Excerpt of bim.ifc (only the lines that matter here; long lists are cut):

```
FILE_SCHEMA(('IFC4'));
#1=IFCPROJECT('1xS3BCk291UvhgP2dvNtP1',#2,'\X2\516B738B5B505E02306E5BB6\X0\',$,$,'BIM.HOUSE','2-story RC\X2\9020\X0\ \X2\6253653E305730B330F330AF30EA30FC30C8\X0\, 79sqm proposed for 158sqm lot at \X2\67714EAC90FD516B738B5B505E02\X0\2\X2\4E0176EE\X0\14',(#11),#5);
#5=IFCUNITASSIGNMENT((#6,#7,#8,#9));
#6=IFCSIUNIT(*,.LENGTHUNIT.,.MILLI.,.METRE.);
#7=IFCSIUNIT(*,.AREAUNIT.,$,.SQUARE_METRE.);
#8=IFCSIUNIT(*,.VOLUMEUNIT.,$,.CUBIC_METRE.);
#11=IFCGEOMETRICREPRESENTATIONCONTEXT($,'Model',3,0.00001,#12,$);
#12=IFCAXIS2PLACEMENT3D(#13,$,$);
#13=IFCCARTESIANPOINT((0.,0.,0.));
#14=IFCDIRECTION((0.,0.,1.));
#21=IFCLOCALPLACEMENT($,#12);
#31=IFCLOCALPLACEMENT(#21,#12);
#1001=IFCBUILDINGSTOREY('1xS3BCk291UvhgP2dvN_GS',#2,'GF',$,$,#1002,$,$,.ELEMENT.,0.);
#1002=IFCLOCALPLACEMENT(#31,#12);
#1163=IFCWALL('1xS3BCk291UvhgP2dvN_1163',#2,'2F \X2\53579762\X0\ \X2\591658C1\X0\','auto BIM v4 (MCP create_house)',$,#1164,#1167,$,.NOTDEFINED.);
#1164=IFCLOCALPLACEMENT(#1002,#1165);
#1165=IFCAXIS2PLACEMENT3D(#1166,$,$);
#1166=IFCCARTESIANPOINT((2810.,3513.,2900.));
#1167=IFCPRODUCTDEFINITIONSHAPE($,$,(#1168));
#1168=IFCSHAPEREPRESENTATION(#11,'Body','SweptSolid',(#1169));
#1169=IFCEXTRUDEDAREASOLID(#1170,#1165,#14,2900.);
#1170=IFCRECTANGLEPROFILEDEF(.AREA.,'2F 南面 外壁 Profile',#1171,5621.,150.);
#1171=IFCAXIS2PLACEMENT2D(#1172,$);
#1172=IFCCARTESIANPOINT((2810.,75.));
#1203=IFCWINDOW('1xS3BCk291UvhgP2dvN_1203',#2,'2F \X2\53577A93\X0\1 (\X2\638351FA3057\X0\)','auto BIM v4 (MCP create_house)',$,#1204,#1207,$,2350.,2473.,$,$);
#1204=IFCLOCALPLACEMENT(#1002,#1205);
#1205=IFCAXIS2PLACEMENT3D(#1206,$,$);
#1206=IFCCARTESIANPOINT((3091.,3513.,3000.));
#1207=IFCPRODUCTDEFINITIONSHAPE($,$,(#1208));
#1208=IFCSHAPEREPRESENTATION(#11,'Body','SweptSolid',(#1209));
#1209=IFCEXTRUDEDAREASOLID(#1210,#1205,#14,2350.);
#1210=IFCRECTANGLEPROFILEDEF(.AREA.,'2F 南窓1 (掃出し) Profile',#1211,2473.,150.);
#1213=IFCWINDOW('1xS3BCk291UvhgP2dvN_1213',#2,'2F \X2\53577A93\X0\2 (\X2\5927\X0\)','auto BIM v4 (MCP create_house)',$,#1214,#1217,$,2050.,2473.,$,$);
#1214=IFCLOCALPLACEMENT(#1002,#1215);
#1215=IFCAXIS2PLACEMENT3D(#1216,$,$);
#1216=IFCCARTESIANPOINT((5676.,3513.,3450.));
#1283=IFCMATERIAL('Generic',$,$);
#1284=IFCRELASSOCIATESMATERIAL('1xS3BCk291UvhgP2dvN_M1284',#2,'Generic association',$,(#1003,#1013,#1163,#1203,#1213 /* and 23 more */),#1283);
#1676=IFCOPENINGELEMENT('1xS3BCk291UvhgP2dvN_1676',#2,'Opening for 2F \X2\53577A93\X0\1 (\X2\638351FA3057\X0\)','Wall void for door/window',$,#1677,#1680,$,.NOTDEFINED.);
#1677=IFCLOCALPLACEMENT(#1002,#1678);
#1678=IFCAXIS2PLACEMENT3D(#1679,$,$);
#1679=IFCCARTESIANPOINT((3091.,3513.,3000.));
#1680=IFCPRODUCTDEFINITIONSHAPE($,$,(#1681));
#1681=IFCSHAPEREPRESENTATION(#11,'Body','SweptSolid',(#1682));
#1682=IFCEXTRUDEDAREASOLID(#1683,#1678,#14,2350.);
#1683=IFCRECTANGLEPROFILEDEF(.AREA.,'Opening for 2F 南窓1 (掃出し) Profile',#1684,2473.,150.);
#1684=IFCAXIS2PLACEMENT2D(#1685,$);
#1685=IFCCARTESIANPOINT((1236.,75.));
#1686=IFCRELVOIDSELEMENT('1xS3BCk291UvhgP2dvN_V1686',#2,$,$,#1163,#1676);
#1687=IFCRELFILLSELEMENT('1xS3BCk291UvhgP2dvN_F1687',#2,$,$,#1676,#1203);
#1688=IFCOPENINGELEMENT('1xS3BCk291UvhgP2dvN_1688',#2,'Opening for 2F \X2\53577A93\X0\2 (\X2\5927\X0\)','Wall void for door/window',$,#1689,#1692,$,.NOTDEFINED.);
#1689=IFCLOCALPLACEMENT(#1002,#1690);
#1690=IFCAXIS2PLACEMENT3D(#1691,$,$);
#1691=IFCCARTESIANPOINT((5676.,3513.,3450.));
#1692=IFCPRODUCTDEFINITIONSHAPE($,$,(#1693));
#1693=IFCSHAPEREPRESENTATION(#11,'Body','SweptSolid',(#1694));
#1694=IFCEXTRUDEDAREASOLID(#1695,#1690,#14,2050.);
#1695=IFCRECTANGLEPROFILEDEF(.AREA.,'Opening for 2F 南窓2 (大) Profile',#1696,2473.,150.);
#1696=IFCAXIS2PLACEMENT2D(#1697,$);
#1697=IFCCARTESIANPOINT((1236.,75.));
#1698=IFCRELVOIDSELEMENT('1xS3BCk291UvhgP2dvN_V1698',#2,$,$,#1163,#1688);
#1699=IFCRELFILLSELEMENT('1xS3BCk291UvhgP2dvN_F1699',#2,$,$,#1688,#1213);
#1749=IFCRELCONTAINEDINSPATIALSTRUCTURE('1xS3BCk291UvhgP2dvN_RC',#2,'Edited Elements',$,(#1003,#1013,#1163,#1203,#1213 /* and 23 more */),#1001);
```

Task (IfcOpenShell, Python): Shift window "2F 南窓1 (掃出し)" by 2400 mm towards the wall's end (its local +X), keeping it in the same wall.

```python
import ifcopenshell
import ifcopenshell.api.geometry
import ifcopenshell.util.placement
import ifcopenshell.util.unit

model = ifcopenshell.open("bim.ifc")
unit_scale = ifcopenshell.util.unit.calculate_unit_scale(model)

window = model.by_guid("1xS3BCk291UvhgP2dvN_1203")
opening = window.FillsVoids[0].RelatingOpeningElement
wall = opening.VoidsElements[0].RelatingBuildingElement

wall_matrix = ifcopenshell.util.placement.get_local_placement(wall.ObjectPlacement)
shift = wall_matrix[:3, 0] * 2.4 / unit_scale
before = ifcopenshell.util.placement.get_local_placement(window.ObjectPlacement)[:3, 3].copy()

# The window is not placed relative to its opening, so move both.
for product in (opening, window):
    matrix = ifcopenshell.util.placement.get_local_placement(product.ObjectPlacement)
    matrix[:3, 3] += shift
    ifcopenshell.api.geometry.edit_object_placement(model, product=product, matrix=matrix, is_si=False)

after = ifcopenshell.util.placement.get_local_placement(window.ObjectPlacement)[:3, 3]
print("window moved by", (after - before).round(3) + 0.0)

model.write("bim_updated.ifc")
```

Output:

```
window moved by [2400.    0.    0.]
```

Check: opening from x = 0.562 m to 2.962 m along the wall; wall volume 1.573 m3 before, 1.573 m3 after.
